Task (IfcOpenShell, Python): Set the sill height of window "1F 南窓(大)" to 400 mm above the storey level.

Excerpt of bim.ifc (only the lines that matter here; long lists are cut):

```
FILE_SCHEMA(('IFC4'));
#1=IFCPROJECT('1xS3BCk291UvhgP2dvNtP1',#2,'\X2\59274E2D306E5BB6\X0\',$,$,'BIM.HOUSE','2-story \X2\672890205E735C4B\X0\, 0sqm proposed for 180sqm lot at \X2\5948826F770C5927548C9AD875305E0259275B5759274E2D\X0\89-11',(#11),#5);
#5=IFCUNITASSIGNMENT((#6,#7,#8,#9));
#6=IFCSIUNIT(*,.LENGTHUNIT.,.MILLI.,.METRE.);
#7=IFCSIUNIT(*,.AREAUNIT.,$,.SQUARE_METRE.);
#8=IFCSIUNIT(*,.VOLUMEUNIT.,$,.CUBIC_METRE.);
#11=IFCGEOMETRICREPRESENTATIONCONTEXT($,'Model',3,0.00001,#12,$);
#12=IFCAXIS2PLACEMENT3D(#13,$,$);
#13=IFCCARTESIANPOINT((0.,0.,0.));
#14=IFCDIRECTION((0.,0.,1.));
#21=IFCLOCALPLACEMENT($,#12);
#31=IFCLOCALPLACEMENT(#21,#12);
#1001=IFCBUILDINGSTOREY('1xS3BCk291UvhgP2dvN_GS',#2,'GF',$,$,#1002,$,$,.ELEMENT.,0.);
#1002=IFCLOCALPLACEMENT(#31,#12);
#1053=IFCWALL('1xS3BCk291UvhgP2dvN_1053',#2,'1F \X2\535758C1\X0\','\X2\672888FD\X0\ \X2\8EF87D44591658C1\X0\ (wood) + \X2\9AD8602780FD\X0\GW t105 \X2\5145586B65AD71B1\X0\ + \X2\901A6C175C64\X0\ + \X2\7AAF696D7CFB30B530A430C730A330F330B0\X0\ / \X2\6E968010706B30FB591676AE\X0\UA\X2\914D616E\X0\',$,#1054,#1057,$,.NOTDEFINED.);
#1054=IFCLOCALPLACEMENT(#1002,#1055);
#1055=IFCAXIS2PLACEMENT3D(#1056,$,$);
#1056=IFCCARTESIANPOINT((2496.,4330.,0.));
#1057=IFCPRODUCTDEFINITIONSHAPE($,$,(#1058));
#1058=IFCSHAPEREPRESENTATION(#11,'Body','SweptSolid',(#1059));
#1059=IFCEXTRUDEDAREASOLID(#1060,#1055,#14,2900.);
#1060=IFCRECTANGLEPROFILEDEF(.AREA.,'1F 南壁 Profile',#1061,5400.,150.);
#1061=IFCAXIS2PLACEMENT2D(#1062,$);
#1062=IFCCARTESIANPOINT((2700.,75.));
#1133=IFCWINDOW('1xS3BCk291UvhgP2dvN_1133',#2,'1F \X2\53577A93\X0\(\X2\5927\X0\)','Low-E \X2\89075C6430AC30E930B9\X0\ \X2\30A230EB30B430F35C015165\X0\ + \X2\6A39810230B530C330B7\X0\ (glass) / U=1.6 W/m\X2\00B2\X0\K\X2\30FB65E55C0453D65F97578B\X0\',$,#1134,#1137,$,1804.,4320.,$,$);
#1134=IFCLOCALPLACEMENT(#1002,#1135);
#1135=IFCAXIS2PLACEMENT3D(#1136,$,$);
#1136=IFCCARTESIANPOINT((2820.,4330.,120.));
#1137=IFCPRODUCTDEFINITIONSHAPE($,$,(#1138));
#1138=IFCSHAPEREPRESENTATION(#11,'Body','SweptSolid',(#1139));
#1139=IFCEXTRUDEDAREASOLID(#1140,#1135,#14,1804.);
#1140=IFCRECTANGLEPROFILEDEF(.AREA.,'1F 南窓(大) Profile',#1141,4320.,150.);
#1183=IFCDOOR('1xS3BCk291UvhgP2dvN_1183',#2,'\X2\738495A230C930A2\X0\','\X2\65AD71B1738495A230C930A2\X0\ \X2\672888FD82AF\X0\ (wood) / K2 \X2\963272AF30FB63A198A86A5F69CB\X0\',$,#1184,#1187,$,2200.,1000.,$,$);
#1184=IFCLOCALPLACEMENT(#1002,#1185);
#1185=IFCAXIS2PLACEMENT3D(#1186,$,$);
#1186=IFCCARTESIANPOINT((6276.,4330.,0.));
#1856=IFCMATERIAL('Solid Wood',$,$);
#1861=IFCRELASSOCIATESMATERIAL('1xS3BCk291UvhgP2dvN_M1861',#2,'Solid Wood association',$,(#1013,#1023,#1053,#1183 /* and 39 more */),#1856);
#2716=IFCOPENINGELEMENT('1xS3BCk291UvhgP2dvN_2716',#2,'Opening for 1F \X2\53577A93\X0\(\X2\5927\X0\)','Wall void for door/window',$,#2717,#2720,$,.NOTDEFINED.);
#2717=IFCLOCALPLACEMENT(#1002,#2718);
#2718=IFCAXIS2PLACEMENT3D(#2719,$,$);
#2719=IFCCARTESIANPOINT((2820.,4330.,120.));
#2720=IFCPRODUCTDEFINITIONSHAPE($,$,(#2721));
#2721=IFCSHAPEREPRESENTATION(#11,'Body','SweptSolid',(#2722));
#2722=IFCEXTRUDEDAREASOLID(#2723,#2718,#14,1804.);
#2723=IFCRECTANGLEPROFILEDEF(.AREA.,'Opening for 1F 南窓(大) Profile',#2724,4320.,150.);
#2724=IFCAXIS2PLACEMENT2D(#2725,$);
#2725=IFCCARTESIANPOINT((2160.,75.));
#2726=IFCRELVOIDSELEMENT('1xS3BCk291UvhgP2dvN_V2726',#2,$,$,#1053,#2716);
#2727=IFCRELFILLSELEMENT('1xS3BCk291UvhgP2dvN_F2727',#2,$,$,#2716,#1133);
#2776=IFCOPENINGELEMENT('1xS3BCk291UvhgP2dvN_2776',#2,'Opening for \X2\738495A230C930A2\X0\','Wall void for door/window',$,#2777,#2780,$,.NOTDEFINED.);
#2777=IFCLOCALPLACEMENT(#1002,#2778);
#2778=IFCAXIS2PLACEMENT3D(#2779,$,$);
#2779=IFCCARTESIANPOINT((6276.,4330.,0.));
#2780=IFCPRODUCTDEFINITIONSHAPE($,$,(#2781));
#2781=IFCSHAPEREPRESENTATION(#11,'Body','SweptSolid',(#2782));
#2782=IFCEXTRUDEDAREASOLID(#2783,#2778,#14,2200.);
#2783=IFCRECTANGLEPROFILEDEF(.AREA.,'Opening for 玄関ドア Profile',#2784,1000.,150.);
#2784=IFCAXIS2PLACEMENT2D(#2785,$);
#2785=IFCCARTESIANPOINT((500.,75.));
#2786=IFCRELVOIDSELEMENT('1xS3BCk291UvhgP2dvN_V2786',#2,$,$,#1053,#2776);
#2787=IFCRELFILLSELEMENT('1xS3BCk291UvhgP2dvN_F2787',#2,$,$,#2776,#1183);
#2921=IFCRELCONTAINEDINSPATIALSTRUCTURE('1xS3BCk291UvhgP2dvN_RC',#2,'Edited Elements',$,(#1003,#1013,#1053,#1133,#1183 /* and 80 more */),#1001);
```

```python
import numpy as np
import ifcopenshell
import ifcopenshell.api.geometry
import ifcopenshell.geom
import ifcopenshell.util.element
import ifcopenshell.util.placement
import ifcopenshell.util.shape
import ifcopenshell.util.unit

model = ifcopenshell.open("bim.ifc")
unit_scale = ifcopenshell.util.unit.calculate_unit_scale(model)

window = model.by_guid("1xS3BCk291UvhgP2dvN_1133")
opening = window.FillsVoids[0].RelatingOpeningElement
storey = ifcopenshell.util.element.get_container(window, ifc_class="IfcBuildingStorey")
level = ifcopenshell.util.placement.get_local_placement(storey.ObjectPlacement)[2, 3]

# The opening's origin need not be at the sill, so measure its lowest point.
shape = ifcopenshell.geom.create_shape(ifcopenshell.geom.settings(), opening)
bottom = ifcopenshell.util.shape.get_shape_bottom_elevation(shape, shape.geometry) / unit_scale
dz = level + 0.4 / unit_scale - bottom

shift = np.array([0.0, 0.0, dz])
# The window is not placed relative to its opening, so move both.
for product in (opening, window):
    matrix = ifcopenshell.util.placement.get_local_placement(product.ObjectPlacement)
    matrix[:3, 3] += shift
    ifcopenshell.api.geometry.edit_object_placement(model, product=product, matrix=matrix, is_si=False)

print(f"moved by {dz * unit_scale:+.3f} m")

model.write("bim_edited.ifc")
```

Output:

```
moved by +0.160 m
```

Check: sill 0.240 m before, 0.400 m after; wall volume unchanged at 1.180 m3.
